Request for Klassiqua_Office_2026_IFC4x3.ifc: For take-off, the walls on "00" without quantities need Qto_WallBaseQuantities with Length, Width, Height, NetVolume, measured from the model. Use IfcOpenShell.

First a look at what the model holds.

```python
import ifcopenshell
import ifcopenshell.util.element
import ifcopenshell.util.unit

model = ifcopenshell.open("Klassiqua_Office_2026_IFC4x3.ifc")
print(model.schema)
for unit_type in ("LENGTHUNIT", "AREAUNIT", "VOLUMEUNIT"):
    print(unit_type, ifcopenshell.util.unit.calculate_unit_scale(model, unit_type))
storey = next(s for s in model.by_type("IfcBuildingStorey") if s.Name == "00")
walls = [e for e in ifcopenshell.util.element.get_decomposition(storey) if e.is_a("IfcWall")]
for e in sorted(walls, key=lambda e: e.id()):
    print(e.id(), e.is_a(), e.Name, list(ifcopenshell.util.element.get_psets(e, qtos_only=True)), sep=" | ")
```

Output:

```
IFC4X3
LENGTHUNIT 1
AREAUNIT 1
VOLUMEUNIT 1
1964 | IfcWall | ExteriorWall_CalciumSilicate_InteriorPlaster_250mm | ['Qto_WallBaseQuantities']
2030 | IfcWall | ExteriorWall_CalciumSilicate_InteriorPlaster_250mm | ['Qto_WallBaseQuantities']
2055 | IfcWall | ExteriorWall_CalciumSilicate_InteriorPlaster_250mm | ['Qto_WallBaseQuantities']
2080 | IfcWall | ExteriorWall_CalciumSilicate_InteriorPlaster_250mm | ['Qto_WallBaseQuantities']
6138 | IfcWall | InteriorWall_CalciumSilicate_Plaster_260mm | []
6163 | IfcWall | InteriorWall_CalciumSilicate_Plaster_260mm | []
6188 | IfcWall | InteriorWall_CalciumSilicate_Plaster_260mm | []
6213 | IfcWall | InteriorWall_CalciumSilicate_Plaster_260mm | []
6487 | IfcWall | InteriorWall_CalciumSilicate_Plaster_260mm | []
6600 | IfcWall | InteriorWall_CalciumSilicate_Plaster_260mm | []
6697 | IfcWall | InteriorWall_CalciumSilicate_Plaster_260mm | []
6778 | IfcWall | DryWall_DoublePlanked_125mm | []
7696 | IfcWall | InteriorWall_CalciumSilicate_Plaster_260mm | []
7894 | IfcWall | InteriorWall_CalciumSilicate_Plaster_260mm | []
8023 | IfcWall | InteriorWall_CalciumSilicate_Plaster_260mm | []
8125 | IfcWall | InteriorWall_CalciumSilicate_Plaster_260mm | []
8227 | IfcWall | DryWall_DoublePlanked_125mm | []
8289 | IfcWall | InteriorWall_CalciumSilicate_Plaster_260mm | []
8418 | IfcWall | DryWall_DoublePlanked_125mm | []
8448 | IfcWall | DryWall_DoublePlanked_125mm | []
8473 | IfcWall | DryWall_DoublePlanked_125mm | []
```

```python
import ifcopenshell
import ifcopenshell.api.pset
import ifcopenshell.geom
import ifcopenshell.util.element
import ifcopenshell.util.shape
import ifcopenshell.util.unit

model = ifcopenshell.open("Klassiqua_Office_2026_IFC4x3.ifc")
unit_scale = ifcopenshell.util.unit.calculate_unit_scale(model)
volume_scale = ifcopenshell.util.unit.calculate_unit_scale(model, "VOLUMEUNIT")
settings = ifcopenshell.geom.settings()

storey = next(s for s in model.by_type("IfcBuildingStorey") if s.Name == "00")
walls = [e for e in ifcopenshell.util.element.get_decomposition(storey) if e.is_a("IfcWall")]

for e in sorted(walls, key=lambda e: e.id()):
    if ifcopenshell.util.element.get_psets(e, qtos_only=True, should_inherit=False):
        continue
    # Geometry comes back in metres, in the element's own axes.
    shape = ifcopenshell.geom.create_shape(settings, e)
    values = {
        "Length": ifcopenshell.util.shape.get_x(shape.geometry) / unit_scale,
        "Width": ifcopenshell.util.shape.get_y(shape.geometry) / unit_scale,
        "Height": ifcopenshell.util.shape.get_z(shape.geometry) / unit_scale,
        "NetVolume": ifcopenshell.util.shape.get_volume(shape.geometry) / volume_scale,
    }
    qto = ifcopenshell.api.pset.add_qto(model, product=e, name="Qto_WallBaseQuantities")
    ifcopenshell.api.pset.edit_qto(model, qto=qto, properties=values)
    print(e.id(), {k: round(v, 3) for k, v in values.items()})

model.write("Klassiqua_Office_2026_IFC4x3_v2.ifc")
```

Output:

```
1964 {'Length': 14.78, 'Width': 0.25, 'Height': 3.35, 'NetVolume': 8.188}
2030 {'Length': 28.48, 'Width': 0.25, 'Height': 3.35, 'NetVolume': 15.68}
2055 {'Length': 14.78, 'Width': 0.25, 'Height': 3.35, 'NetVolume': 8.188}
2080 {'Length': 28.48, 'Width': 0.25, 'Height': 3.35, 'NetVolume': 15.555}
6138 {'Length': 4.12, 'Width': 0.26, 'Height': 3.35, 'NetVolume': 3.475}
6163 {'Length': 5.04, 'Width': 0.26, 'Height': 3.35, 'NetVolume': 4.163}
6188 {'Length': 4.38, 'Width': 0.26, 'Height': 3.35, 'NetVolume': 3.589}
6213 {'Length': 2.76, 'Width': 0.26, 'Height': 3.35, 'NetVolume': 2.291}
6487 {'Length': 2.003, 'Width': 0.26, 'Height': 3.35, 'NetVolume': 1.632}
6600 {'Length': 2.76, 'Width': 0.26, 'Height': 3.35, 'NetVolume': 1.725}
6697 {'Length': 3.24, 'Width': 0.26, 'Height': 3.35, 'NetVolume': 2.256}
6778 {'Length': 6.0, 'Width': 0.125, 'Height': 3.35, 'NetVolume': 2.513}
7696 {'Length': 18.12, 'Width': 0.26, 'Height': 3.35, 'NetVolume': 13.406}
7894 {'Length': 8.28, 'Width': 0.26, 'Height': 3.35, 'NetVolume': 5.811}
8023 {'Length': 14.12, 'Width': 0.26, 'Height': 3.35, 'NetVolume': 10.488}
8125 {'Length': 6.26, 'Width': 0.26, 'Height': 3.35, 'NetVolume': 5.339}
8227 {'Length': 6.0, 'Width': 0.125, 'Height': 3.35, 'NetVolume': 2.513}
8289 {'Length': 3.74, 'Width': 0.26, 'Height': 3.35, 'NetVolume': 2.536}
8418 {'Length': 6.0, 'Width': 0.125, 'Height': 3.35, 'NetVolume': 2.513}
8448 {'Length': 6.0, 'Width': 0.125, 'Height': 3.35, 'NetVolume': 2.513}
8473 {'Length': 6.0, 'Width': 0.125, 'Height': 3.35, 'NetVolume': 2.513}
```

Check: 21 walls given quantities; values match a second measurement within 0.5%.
